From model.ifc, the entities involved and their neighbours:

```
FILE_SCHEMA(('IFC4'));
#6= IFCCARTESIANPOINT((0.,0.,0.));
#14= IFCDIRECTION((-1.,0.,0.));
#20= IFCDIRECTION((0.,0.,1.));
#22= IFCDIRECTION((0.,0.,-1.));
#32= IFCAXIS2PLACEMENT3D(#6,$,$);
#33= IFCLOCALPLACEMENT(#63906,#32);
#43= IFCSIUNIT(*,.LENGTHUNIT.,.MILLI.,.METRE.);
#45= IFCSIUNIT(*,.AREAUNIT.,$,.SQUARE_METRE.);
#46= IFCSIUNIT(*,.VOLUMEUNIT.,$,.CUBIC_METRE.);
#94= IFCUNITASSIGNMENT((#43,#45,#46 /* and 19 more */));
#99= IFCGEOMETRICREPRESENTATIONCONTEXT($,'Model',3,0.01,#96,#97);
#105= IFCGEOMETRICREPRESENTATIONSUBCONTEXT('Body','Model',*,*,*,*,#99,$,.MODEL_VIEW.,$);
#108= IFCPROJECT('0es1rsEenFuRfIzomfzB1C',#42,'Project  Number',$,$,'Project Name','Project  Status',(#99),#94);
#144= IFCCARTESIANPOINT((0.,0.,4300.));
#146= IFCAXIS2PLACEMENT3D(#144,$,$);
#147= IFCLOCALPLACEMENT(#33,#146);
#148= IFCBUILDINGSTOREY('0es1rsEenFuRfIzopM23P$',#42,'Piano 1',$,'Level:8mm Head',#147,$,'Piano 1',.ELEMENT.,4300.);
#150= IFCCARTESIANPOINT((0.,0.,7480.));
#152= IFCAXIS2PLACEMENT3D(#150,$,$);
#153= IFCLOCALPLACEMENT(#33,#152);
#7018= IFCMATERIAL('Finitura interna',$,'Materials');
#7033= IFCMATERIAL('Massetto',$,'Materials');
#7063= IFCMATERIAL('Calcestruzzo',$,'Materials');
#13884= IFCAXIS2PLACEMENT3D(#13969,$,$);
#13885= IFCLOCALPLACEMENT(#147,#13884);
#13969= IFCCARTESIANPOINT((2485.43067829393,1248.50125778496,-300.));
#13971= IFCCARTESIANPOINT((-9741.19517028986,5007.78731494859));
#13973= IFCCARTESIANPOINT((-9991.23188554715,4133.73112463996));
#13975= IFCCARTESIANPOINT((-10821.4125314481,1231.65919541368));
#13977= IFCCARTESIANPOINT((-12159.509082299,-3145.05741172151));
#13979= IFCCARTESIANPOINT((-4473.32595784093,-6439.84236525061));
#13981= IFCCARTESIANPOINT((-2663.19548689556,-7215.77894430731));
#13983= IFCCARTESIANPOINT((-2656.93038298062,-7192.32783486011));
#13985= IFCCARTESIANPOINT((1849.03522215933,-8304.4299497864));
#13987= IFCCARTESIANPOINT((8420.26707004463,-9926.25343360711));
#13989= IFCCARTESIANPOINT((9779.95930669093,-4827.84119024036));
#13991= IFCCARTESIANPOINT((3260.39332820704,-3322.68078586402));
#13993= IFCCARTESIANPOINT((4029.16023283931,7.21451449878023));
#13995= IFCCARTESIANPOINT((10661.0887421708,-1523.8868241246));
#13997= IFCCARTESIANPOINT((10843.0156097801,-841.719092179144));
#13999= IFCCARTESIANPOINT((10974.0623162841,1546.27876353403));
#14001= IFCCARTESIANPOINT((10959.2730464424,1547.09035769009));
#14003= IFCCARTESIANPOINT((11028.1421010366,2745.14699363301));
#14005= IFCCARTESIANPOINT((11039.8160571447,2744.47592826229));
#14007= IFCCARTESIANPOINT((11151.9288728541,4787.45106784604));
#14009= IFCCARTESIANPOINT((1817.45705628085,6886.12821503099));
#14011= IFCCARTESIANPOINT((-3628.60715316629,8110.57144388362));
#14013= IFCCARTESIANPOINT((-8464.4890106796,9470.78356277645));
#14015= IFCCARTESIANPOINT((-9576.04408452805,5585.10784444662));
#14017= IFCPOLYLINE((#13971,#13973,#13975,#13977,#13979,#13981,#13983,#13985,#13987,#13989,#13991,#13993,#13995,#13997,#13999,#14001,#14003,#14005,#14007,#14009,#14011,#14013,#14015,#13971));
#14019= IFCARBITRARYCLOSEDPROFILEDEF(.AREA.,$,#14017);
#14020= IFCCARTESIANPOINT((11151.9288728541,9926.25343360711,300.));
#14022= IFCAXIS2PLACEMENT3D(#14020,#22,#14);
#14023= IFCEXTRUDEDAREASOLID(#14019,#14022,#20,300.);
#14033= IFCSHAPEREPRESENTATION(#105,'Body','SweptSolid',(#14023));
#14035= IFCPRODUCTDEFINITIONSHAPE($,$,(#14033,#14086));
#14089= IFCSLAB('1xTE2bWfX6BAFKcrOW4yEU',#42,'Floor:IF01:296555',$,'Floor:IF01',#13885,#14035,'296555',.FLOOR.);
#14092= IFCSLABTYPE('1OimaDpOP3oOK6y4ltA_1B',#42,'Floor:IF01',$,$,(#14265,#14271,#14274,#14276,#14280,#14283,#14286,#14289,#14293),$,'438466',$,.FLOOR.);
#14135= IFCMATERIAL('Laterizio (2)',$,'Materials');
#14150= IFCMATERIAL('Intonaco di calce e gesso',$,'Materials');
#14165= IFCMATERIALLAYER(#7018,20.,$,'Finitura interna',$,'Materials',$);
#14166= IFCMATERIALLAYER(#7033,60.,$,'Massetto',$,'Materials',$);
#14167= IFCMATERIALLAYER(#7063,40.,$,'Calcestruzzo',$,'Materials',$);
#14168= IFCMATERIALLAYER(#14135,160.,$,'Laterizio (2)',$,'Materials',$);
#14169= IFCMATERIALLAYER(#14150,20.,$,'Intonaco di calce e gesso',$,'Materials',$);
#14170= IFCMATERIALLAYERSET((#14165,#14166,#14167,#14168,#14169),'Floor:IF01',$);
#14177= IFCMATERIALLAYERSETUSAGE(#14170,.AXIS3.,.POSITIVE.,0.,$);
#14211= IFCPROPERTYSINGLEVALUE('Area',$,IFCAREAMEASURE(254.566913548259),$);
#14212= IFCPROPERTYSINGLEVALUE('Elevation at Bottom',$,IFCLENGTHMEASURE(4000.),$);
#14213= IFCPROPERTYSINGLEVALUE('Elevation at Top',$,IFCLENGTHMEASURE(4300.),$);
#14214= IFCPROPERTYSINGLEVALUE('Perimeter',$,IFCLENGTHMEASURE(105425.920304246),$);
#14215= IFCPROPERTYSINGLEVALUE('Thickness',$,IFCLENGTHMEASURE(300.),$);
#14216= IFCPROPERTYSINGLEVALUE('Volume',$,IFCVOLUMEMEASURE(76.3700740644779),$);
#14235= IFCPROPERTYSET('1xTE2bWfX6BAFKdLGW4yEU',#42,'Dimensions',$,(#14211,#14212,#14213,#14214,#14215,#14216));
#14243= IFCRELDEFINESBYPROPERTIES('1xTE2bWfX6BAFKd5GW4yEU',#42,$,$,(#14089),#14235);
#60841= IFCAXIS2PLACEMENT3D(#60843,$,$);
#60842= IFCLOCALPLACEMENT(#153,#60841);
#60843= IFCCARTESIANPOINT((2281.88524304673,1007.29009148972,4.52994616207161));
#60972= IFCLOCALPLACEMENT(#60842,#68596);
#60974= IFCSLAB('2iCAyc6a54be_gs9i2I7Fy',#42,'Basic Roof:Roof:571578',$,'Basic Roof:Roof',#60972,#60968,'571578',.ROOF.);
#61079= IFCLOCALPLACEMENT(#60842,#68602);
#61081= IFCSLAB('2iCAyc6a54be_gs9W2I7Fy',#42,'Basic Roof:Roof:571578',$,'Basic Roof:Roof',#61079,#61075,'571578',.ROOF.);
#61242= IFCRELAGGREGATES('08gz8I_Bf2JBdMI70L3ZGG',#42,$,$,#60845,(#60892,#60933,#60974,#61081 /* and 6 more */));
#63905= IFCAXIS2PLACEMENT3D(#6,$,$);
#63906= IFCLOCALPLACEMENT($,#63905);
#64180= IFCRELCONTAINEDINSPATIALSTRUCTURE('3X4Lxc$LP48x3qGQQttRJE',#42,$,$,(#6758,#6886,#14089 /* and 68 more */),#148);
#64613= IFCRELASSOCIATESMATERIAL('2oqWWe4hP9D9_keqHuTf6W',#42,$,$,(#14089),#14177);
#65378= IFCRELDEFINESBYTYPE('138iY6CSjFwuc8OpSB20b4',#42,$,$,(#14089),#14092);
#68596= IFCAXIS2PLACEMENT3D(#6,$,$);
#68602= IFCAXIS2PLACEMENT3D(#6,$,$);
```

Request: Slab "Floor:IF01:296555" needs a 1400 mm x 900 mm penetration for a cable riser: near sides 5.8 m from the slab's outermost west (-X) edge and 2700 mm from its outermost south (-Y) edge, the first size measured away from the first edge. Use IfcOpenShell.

```python
import numpy as np
import ifcopenshell
import ifcopenshell.api.feature
import ifcopenshell.api.geometry
import ifcopenshell.api.pset
import ifcopenshell.api.root
import ifcopenshell.geom
import ifcopenshell.util.element
import ifcopenshell.util.placement
import ifcopenshell.util.representation
import ifcopenshell.util.shape
import ifcopenshell.util.unit

model = ifcopenshell.open("model.ifc")
unit_scale = ifcopenshell.util.unit.calculate_unit_scale(model)
area_scale = ifcopenshell.util.unit.calculate_unit_scale(model, "AREAUNIT")
volume_scale = ifcopenshell.util.unit.calculate_unit_scale(model, "VOLUMEUNIT")
settings = ifcopenshell.geom.settings()


def volume(element):
    """Net volume in cubic metres, openings subtracted."""
    shape = ifcopenshell.geom.create_shape(settings, element)
    return ifcopenshell.util.shape.get_volume(shape.geometry)


slab = model.by_id(14089)
before = volume(slab)

# Extent in the slab's own axes, in metres. The edges named are its -X and -Y sides.
slab_shape = ifcopenshell.geom.create_shape(settings, slab)
vertices = ifcopenshell.util.shape.get_vertices(slab_shape.geometry)
x_min, y_min, bottom = vertices.min(axis=0)
top = vertices[:, 2].max()

opening = ifcopenshell.api.root.create_entity(model, ifc_class="IfcOpeningElement", name="Cable riser opening", predefined_type="OPENING")
context = ifcopenshell.util.representation.get_context(model, "Model", "Body", "MODEL_VIEW")
width, depth = 1.4, 0.9
outline = [(0.0, 0.0), (width, 0.0), (width, depth), (0.0, depth), (0.0, 0.0)]
# Overshoot both faces by 50 mm so the cut is clean.
shape = ifcopenshell.api.geometry.add_slab_representation(
    model, context=context, depth=top - bottom + 0.1, polyline=outline
)
ifcopenshell.api.geometry.assign_representation(model, product=opening, representation=shape)

matrix = ifcopenshell.util.placement.get_local_placement(slab.ObjectPlacement)
matrix[:, 3] = matrix @ np.append(np.array([x_min + 5.8, y_min + 2.7, bottom - 0.05]) / unit_scale, 1.0)
ifcopenshell.api.geometry.edit_object_placement(model, product=opening, matrix=matrix, is_si=False)
ifcopenshell.api.feature.add_feature(model, feature=opening, element=slab)

after = volume(slab)

# Update the slab's stored quantities.
pset = model.by_id(ifcopenshell.util.element.get_pset(slab, "Dimensions", should_inherit=False)["id"])
ifcopenshell.api.pset.edit_pset(model, pset=pset, properties={
    "Area": model.create_entity("IfcAreaMeasure", after / (top - bottom) / area_scale),
    "Volume": model.create_entity("IfcVolumeMeasure", after / volume_scale),
})

print(f"slab volume {before:.3f} -> {after:.3f} m3")

model.write("model_updated.ifc")
```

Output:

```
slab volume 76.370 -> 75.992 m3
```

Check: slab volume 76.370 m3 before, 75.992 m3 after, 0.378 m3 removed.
